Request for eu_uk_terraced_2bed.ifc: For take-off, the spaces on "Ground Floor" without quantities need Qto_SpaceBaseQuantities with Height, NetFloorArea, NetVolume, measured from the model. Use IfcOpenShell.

First a look at what the model holds.

```python
import ifcopenshell
import ifcopenshell.util.element
import ifcopenshell.util.unit

model = ifcopenshell.open("eu_uk_terraced_2bed.ifc")
print(model.schema)
for unit_type in ("LENGTHUNIT", "AREAUNIT", "VOLUMEUNIT"):
    print(unit_type, ifcopenshell.util.unit.calculate_unit_scale(model, unit_type))
storey = next(s for s in model.by_type("IfcBuildingStorey") if s.Name == "Ground Floor")
spaces = [e for e in ifcopenshell.util.element.get_decomposition(storey) if e.is_a("IfcSpace")]
for e in sorted(spaces, key=lambda e: e.id()):
    print(e.id(), e.is_a(), e.Name, list(ifcopenshell.util.element.get_psets(e, qtos_only=True)), sep=" | ")
```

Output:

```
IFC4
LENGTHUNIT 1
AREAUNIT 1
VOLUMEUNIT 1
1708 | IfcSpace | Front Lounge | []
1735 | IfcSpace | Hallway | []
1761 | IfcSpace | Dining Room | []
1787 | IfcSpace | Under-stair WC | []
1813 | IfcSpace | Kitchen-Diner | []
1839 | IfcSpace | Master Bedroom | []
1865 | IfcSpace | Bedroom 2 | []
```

```python
import ifcopenshell
import ifcopenshell.api.pset
import ifcopenshell.geom
import ifcopenshell.util.element
import ifcopenshell.util.shape
import ifcopenshell.util.unit

model = ifcopenshell.open("eu_uk_terraced_2bed.ifc")
unit_scale = ifcopenshell.util.unit.calculate_unit_scale(model)
area_scale = ifcopenshell.util.unit.calculate_unit_scale(model, "AREAUNIT")
volume_scale = ifcopenshell.util.unit.calculate_unit_scale(model, "VOLUMEUNIT")
settings = ifcopenshell.geom.settings()

storey = next(s for s in model.by_type("IfcBuildingStorey") if s.Name == "Ground Floor")
spaces = [e for e in ifcopenshell.util.element.get_decomposition(storey) if e.is_a("IfcSpace")]

for e in sorted(spaces, key=lambda e: e.id()):
    if ifcopenshell.util.element.get_psets(e, qtos_only=True, should_inherit=False):
        continue
    # Geometry comes back in metres, in the element's own axes.
    shape = ifcopenshell.geom.create_shape(settings, e)
    values = {
        "Height": ifcopenshell.util.shape.get_z(shape.geometry) / unit_scale,
        "NetFloorArea": ifcopenshell.util.shape.get_footprint_area(shape.geometry) / area_scale,
        "NetVolume": ifcopenshell.util.shape.get_volume(shape.geometry) / volume_scale,
    }
    qto = ifcopenshell.api.pset.add_qto(model, product=e, name="Qto_SpaceBaseQuantities")
    ifcopenshell.api.pset.edit_qto(model, qto=qto, properties=values)
    print(e.id(), {k: round(v, 3) for k, v in values.items()})

model.write("eu_uk_terraced_2bed_edited.ifc")
```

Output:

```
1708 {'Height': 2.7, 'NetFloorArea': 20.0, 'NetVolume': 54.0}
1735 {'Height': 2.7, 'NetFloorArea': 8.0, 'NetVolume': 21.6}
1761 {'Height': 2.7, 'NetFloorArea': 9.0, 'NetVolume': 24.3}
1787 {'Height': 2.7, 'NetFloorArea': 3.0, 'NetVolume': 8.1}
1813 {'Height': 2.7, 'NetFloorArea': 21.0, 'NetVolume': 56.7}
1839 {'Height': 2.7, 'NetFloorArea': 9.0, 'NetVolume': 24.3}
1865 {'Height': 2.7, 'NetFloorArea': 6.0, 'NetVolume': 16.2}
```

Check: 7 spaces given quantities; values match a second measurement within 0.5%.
